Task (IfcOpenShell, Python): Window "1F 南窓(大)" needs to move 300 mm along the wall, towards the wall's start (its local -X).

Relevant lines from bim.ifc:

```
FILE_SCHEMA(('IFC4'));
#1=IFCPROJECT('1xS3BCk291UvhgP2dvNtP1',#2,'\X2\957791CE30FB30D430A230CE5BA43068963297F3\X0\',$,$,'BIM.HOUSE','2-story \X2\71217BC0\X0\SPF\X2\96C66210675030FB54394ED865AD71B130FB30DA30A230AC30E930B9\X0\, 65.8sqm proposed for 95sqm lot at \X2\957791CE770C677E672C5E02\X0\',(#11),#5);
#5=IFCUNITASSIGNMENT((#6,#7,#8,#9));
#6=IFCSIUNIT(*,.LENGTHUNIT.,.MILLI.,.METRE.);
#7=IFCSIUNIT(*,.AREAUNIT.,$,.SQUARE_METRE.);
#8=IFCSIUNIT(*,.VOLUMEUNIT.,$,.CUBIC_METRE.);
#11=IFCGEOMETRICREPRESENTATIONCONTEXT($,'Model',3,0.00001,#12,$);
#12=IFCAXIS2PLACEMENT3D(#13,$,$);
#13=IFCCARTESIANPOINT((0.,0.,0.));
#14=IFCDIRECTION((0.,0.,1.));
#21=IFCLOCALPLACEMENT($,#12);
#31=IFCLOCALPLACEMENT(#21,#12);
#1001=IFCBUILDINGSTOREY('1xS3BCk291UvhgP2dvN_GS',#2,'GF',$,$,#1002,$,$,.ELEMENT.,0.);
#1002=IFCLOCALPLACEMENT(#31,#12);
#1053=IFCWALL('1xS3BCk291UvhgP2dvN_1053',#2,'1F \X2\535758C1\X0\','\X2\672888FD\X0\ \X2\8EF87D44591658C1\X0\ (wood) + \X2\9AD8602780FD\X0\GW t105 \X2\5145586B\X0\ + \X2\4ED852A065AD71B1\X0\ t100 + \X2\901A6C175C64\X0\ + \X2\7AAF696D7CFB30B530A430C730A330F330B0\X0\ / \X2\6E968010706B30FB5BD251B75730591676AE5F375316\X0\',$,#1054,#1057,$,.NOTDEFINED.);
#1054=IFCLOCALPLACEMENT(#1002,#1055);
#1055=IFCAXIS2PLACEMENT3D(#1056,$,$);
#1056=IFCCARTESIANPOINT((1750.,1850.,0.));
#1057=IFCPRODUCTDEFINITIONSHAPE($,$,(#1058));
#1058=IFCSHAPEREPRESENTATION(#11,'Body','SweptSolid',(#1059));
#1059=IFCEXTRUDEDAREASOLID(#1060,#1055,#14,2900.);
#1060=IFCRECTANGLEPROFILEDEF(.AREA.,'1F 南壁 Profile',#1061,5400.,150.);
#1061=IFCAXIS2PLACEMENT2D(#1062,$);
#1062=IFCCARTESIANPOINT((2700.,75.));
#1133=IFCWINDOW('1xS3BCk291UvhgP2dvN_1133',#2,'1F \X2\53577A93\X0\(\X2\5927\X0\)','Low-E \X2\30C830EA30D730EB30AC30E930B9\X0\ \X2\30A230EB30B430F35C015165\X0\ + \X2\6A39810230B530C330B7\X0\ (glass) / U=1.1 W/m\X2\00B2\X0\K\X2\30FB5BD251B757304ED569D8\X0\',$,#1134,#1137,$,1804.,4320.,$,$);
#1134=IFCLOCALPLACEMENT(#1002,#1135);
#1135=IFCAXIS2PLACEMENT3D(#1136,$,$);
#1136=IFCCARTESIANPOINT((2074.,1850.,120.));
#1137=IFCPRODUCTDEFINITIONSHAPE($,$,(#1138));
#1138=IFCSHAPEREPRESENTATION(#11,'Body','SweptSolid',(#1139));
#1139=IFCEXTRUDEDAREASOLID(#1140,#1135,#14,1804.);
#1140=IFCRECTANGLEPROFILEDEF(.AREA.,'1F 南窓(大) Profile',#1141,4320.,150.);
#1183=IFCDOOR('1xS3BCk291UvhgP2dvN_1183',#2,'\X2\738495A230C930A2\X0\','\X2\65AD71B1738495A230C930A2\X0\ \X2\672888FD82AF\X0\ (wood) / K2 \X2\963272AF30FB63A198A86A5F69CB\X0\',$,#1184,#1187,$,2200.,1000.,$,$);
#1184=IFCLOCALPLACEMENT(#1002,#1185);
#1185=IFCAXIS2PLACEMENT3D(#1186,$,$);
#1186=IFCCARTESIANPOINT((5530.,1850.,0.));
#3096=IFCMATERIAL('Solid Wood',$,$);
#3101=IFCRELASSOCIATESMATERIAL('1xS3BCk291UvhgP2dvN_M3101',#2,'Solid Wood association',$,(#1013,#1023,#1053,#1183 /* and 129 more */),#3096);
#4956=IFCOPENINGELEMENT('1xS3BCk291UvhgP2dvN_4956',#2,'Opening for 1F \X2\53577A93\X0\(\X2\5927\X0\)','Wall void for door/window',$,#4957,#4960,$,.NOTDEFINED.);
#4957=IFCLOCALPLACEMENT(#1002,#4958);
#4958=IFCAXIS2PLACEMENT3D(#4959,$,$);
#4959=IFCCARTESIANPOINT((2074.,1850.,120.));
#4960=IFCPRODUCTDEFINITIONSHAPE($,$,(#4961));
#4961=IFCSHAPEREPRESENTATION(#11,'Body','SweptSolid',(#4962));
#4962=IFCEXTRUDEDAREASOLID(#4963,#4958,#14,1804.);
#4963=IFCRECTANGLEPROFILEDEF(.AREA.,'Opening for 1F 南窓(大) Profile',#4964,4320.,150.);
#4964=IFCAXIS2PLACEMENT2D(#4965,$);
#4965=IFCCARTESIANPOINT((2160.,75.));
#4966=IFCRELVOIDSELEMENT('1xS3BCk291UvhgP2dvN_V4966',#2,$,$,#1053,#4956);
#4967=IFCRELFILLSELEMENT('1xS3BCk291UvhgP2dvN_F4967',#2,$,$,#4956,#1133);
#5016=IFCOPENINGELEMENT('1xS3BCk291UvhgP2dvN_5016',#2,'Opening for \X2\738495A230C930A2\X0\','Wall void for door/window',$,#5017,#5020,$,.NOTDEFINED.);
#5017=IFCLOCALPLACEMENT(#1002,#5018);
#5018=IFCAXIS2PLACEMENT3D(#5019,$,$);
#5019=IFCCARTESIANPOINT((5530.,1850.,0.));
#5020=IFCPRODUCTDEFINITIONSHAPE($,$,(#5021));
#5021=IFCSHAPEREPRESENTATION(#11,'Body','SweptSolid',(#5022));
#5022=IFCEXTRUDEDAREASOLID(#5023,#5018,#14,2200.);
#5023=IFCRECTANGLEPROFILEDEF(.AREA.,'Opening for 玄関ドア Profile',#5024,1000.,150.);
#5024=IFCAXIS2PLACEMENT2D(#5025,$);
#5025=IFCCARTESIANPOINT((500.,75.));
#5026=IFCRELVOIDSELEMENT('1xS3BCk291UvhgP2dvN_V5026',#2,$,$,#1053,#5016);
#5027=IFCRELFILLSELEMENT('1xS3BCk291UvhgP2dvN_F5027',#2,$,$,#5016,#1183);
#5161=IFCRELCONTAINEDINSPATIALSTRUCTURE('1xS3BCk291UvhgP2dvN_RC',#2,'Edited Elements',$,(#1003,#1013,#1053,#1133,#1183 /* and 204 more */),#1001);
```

```python
import ifcopenshell
import ifcopenshell.api.geometry
import ifcopenshell.util.placement

model = ifcopenshell.open("bim.ifc")

window = model.by_guid("1xS3BCk291UvhgP2dvN_1133")
opening = window.FillsVoids[0].RelatingOpeningElement
wall = opening.VoidsElements[0].RelatingBuildingElement

wall_matrix = ifcopenshell.util.placement.get_local_placement(wall.ObjectPlacement)
shift = wall_matrix[:3, 0] * -300.0
before = ifcopenshell.util.placement.get_local_placement(window.ObjectPlacement)[:3, 3].copy()

# The window is not placed relative to its opening, so move both.
for product in (opening, window):
    matrix = ifcopenshell.util.placement.get_local_placement(product.ObjectPlacement)
    matrix[:3, 3] += shift
    ifcopenshell.api.geometry.edit_object_placement(model, product=product, matrix=matrix, is_si=False)

after = ifcopenshell.util.placement.get_local_placement(window.ObjectPlacement)[:3, 3]
print("window moved by", (after - before).round(3) + 0.0)

model.write("bim_v2.ifc")
```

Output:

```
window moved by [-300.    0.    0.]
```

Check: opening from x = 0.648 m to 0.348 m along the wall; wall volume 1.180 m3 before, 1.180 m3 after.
